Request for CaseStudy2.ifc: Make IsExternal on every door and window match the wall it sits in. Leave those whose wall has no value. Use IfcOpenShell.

First a look at what the model holds.

```python
import ifcopenshell
import ifcopenshell.util.element

model = ifcopenshell.open("CaseStudy2.ifc")
print(model.schema)
seen = {}
for e in model.by_type("IfcDoor") + model.by_type("IfcWindow"):
    if not e.FillsVoids:
        continue
    host = e.FillsVoids[0].RelatingOpeningElement.VoidsElements[0].RelatingBuildingElement
    own = ifcopenshell.util.element.get_pset(e, f"Pset_{e.is_a()[3:].removesuffix('StandardCase')}Common", "IsExternal")
    wall = ifcopenshell.util.element.get_pset(host, "Pset_WallCommon", "IsExternal")
    seen[e.is_a(), own, wall] = seen.get((e.is_a(), own, wall), 0) + 1
for (cls, own, wall), count in sorted(seen.items(), key=str):
    print(count, cls, "IsExternal:", own, "| host wall:", wall)
```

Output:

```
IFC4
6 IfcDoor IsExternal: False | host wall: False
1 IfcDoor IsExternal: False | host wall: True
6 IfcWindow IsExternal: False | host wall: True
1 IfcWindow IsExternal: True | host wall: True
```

```python
import ifcopenshell
import ifcopenshell.api.pset
import ifcopenshell.util.element

model = ifcopenshell.open("CaseStudy2.ifc")

count = 0
for ifc_class, pset_name in (("IfcDoor", "Pset_DoorCommon"), ("IfcWindow", "Pset_WindowCommon")):
    for e in model.by_type(ifc_class):
        if not e.FillsVoids:
            continue
        host = e.FillsVoids[0].RelatingOpeningElement.VoidsElements[0].RelatingBuildingElement
        external = ifcopenshell.util.element.get_pset(host, "Pset_WallCommon", "IsExternal")
        if external is None or ifcopenshell.util.element.get_pset(e, pset_name, "IsExternal") == external:
            continue
        pset = ifcopenshell.api.pset.add_pset(model, product=e, name=pset_name)
        ifcopenshell.api.pset.edit_pset(model, pset=pset, properties={"IsExternal": external})
        count += 1

print(count, "updated")

model.write("CaseStudy2_rev.ifc")
```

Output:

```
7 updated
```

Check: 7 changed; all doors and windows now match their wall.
